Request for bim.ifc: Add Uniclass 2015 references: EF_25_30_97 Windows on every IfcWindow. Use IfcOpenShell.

First a look at what the model holds.

```python
import ifcopenshell

model = ifcopenshell.open("bim.ifc")
print(model.schema)
print("classifications:", [c.Name for c in model.by_type("IfcClassification")])
for ifc_class in ("IfcDoor", "IfcRoof", "IfcStair", "IfcWall", "IfcWindow"):
    print(ifc_class, len(model.by_type(ifc_class)))
```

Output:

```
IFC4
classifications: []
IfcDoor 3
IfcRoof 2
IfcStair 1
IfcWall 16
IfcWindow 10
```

```python
import ifcopenshell
import ifcopenshell.api.classification

model = ifcopenshell.open("bim.ifc")

system = ifcopenshell.api.classification.add_classification(model, classification="Uniclass 2015")

codes = {
    "IfcWindow": ("EF_25_30_97", "Windows"),
}
for ifc_class, (code, name) in codes.items():
    products = model.by_type(ifc_class)
    ifcopenshell.api.classification.add_reference(
        model, products=products, classification=system, identification=code, name=name
    )
    print(code, len(products))

model.write("bim_rev.ifc")
```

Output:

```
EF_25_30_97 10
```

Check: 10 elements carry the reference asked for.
